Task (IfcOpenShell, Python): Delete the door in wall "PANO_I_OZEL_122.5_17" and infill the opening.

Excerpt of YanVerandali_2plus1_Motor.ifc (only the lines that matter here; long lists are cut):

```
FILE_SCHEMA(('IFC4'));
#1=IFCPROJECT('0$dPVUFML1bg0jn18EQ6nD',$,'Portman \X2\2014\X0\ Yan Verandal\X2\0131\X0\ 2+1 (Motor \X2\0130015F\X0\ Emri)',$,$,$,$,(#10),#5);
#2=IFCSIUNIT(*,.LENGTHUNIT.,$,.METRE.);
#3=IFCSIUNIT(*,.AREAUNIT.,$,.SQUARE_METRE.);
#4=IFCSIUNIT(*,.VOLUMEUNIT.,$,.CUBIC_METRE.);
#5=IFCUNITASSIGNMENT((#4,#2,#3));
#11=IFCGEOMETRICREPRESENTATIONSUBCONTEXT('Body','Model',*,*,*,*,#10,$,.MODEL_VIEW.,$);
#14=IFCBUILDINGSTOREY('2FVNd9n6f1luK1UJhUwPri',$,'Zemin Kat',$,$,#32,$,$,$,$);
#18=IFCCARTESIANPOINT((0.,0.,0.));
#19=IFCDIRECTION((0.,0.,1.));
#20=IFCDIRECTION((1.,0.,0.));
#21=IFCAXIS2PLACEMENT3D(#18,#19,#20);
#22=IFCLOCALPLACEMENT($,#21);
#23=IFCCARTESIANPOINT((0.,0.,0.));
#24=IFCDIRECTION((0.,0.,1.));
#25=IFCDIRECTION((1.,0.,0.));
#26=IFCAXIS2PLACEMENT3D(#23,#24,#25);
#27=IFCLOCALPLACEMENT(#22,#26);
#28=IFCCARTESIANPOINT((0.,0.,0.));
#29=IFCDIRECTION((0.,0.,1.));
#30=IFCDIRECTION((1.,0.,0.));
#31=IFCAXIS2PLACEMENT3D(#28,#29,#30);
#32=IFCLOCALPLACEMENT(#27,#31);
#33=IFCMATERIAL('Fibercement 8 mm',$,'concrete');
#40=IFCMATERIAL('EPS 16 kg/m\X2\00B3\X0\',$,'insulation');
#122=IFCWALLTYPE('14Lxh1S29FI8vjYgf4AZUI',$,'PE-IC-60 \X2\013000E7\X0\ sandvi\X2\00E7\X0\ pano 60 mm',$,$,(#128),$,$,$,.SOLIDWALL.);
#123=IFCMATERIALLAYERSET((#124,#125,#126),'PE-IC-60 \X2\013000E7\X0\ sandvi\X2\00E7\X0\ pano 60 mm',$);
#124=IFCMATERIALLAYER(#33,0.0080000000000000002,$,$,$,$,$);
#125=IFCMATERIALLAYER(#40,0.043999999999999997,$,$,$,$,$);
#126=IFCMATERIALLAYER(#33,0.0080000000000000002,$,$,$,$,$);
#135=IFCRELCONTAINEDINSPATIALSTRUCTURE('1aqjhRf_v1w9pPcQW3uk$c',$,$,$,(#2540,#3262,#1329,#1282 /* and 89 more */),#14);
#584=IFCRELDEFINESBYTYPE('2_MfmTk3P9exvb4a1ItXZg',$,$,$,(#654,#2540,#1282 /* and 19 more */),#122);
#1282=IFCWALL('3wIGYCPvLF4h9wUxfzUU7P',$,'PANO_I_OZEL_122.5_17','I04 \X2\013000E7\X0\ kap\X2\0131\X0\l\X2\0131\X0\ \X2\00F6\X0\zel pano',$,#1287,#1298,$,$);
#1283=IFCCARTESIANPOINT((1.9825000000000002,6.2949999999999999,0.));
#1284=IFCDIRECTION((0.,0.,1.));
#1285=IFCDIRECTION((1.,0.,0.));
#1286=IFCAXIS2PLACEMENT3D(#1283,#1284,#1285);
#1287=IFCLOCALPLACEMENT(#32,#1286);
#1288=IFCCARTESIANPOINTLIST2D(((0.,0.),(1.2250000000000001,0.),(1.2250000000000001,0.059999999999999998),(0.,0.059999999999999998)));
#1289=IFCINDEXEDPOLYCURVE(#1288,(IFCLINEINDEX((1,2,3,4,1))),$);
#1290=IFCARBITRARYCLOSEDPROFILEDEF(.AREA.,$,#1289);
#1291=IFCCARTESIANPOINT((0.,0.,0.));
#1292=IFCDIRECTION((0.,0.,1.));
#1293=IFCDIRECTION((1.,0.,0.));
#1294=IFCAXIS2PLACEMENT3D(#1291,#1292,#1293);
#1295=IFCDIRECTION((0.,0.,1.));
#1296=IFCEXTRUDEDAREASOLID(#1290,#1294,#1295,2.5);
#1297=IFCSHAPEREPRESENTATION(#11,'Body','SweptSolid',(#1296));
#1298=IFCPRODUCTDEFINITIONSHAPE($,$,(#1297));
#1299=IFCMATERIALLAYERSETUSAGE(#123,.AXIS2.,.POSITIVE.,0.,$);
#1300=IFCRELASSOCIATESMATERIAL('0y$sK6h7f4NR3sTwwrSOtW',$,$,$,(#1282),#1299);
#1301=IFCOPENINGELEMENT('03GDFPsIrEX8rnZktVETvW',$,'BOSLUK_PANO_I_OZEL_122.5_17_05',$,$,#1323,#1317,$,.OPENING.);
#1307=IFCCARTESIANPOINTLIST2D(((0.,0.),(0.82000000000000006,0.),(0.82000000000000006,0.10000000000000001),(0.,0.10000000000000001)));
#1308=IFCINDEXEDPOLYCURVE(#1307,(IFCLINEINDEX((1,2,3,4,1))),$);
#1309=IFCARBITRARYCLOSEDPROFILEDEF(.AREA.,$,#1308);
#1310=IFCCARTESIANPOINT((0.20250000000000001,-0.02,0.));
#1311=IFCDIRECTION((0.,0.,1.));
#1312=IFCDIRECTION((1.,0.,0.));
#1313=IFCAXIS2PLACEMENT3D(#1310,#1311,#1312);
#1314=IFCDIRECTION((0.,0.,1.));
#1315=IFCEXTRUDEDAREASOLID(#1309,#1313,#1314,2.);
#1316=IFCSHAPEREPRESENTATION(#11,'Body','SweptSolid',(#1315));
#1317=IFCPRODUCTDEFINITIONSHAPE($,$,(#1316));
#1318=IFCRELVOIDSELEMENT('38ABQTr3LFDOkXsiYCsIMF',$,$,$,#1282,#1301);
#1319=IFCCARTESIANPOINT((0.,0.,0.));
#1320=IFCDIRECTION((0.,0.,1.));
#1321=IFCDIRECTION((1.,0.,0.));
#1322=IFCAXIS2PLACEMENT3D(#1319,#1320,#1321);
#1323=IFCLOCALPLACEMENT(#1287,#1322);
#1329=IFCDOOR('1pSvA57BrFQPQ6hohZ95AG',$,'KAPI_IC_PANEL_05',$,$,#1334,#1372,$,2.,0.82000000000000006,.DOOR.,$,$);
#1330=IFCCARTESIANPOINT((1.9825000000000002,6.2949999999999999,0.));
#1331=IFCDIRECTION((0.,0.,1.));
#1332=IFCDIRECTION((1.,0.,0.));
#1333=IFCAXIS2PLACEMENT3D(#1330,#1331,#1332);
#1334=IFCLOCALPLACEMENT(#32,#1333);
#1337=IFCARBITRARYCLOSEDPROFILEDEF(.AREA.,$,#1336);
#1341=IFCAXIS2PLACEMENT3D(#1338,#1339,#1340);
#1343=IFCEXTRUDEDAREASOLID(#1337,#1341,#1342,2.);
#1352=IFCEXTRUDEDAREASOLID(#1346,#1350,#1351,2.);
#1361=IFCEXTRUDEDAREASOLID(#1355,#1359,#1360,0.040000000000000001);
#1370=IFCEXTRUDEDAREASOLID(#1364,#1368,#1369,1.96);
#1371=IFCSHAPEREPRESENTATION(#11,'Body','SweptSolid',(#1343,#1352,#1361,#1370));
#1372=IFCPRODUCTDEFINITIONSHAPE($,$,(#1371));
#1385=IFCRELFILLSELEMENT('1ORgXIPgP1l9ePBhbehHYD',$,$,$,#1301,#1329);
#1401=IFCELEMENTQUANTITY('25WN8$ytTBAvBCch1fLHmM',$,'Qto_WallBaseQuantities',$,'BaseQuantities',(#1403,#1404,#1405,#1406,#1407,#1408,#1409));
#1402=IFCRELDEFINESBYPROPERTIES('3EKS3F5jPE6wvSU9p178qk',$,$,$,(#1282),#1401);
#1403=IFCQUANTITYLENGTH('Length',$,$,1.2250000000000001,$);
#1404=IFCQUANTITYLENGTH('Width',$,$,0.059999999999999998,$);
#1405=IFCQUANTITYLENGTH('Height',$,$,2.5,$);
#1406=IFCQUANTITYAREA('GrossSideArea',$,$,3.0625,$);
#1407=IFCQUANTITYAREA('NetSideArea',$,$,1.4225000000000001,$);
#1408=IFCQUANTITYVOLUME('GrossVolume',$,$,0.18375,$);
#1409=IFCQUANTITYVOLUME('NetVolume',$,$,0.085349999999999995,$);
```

```python
import ifcopenshell
import ifcopenshell.api.feature
import ifcopenshell.api.pset
import ifcopenshell.api.root
import ifcopenshell.geom
import ifcopenshell.util.element
import ifcopenshell.util.shape
import ifcopenshell.util.unit

model = ifcopenshell.open("YanVerandali_2plus1_Motor.ifc")
area_scale = ifcopenshell.util.unit.calculate_unit_scale(model, "AREAUNIT")
volume_scale = ifcopenshell.util.unit.calculate_unit_scale(model, "VOLUMEUNIT")
settings = ifcopenshell.geom.settings()


def volume(element):
    """Net volume in cubic metres, openings subtracted."""
    shape = ifcopenshell.geom.create_shape(settings, element)
    return ifcopenshell.util.shape.get_volume(shape.geometry)


door = model.by_guid("1pSvA57BrFQPQ6hohZ95AG")
opening = door.FillsVoids[0].RelatingOpeningElement
wall = opening.VoidsElements[0].RelatingBuildingElement
before = volume(wall)

ifcopenshell.api.root.remove_product(model, product=door)
ifcopenshell.api.feature.remove_feature(model, feature=opening)

after = volume(wall)
thickness = 0.06  # wall thickness in metres

# Update the wall's stored quantities.
qto = model.by_id(ifcopenshell.util.element.get_pset(wall, "Qto_WallBaseQuantities", should_inherit=False)["id"])
ifcopenshell.api.pset.edit_qto(model, qto=qto, properties={
    "NetSideArea": after / thickness / area_scale,
    "NetVolume": after / volume_scale,
})

print(f"wall volume {before:.3f} -> {after:.3f} m3")

model.write("YanVerandali_2plus1_Motor_updated.ifc")
```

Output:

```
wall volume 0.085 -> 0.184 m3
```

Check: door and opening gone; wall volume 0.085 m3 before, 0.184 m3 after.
